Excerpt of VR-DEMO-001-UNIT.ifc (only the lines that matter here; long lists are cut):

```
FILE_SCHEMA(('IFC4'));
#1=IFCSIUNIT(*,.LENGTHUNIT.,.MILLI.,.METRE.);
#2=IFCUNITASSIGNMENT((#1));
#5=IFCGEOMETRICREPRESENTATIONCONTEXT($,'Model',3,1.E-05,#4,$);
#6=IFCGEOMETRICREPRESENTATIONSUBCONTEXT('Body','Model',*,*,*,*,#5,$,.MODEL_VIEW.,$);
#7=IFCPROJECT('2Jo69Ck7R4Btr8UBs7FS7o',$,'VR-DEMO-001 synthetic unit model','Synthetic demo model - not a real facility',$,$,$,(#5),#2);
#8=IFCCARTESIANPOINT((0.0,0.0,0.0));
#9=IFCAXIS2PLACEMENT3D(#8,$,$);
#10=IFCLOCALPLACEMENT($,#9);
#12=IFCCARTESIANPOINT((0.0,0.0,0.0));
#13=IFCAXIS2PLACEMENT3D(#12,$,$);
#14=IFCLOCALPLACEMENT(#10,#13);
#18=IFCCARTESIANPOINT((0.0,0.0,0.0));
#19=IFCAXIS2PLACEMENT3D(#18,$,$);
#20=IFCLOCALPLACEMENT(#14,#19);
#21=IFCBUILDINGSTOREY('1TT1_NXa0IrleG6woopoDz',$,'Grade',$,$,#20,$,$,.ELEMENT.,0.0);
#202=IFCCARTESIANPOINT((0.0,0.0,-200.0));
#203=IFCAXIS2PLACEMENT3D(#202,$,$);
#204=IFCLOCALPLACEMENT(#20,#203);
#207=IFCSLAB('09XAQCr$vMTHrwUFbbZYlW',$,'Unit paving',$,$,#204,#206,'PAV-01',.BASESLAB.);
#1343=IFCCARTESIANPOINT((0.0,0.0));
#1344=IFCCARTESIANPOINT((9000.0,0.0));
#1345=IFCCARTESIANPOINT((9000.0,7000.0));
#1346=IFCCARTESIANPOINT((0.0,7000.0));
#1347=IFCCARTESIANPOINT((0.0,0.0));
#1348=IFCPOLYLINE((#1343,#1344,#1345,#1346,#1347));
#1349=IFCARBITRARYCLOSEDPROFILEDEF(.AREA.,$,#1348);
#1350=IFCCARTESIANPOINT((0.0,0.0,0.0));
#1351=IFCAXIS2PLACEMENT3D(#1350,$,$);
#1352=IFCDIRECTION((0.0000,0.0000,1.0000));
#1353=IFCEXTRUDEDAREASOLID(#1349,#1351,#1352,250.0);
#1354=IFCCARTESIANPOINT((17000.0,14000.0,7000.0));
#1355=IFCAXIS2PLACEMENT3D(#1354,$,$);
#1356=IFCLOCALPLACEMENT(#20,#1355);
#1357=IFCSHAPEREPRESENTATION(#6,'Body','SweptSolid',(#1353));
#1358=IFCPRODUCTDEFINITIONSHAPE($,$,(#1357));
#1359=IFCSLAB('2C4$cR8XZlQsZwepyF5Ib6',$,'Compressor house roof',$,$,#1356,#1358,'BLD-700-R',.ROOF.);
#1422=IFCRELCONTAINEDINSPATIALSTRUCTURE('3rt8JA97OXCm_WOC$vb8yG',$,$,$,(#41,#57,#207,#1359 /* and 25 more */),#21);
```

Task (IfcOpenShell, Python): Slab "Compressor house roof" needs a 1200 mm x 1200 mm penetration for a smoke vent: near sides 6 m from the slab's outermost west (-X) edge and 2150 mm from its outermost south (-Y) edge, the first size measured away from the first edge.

```python
import numpy as np
import ifcopenshell
import ifcopenshell.api.feature
import ifcopenshell.api.geometry
import ifcopenshell.api.root
import ifcopenshell.geom
import ifcopenshell.util.placement
import ifcopenshell.util.representation
import ifcopenshell.util.shape
import ifcopenshell.util.unit

model = ifcopenshell.open("VR-DEMO-001-UNIT.ifc")
unit_scale = ifcopenshell.util.unit.calculate_unit_scale(model)
settings = ifcopenshell.geom.settings()


def volume(element):
    """Net volume in cubic metres, openings subtracted."""
    shape = ifcopenshell.geom.create_shape(settings, element)
    return ifcopenshell.util.shape.get_volume(shape.geometry)


slab = model.by_guid("2C4$cR8XZlQsZwepyF5Ib6")
before = volume(slab)

# Extent in the slab's own axes, in metres. The edges named are its -X and -Y sides.
slab_shape = ifcopenshell.geom.create_shape(settings, slab)
vertices = ifcopenshell.util.shape.get_vertices(slab_shape.geometry)
x_min, y_min, bottom = vertices.min(axis=0)
top = vertices[:, 2].max()

opening = ifcopenshell.api.root.create_entity(model, ifc_class="IfcOpeningElement", name="Smoke vent opening", predefined_type="OPENING")
context = ifcopenshell.util.representation.get_context(model, "Model", "Body", "MODEL_VIEW")
width, depth = 1.2, 1.2
outline = [(0.0, 0.0), (width, 0.0), (width, depth), (0.0, depth), (0.0, 0.0)]
# Overshoot both faces by 50 mm so the cut is clean.
shape = ifcopenshell.api.geometry.add_slab_representation(
    model, context=context, depth=top - bottom + 0.1, polyline=outline
)
ifcopenshell.api.geometry.assign_representation(model, product=opening, representation=shape)

matrix = ifcopenshell.util.placement.get_local_placement(slab.ObjectPlacement)
matrix[:, 3] = matrix @ np.append(np.array([x_min + 6, y_min + 2.15, bottom - 0.05]) / unit_scale, 1.0)
ifcopenshell.api.geometry.edit_object_placement(model, product=opening, matrix=matrix, is_si=False)
ifcopenshell.api.feature.add_feature(model, feature=opening, element=slab)

after = volume(slab)

print(f"slab volume {before:.3f} -> {after:.3f} m3")

model.write("VR-DEMO-001-UNIT_updated.ifc")
```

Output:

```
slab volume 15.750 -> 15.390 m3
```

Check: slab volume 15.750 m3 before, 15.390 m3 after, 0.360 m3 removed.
